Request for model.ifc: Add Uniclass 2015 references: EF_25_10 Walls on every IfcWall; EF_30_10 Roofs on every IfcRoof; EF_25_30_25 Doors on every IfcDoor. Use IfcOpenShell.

First a look at what the model holds.

```python
import ifcopenshell

model = ifcopenshell.open("model.ifc")
print(model.schema)
print("classifications:", [c.Name for c in model.by_type("IfcClassification")])
for ifc_class in ("IfcDoor", "IfcRoof", "IfcStair", "IfcWall", "IfcWindow"):
    print(ifc_class, len(model.by_type(ifc_class)))
```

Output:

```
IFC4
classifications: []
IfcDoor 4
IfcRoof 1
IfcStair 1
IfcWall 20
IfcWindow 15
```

```python
import ifcopenshell
import ifcopenshell.api.classification

model = ifcopenshell.open("model.ifc")

system = ifcopenshell.api.classification.add_classification(model, classification="Uniclass 2015")

codes = {
    "IfcWall": ("EF_25_10", "Walls"),
    "IfcRoof": ("EF_30_10", "Roofs"),
    "IfcDoor": ("EF_25_30_25", "Doors"),
}
for ifc_class, (code, name) in codes.items():
    products = model.by_type(ifc_class)
    ifcopenshell.api.classification.add_reference(
        model, products=products, classification=system, identification=code, name=name
    )
    print(code, len(products))

model.write("model_updated.ifc")
```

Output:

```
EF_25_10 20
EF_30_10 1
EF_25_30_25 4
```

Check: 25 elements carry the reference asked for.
